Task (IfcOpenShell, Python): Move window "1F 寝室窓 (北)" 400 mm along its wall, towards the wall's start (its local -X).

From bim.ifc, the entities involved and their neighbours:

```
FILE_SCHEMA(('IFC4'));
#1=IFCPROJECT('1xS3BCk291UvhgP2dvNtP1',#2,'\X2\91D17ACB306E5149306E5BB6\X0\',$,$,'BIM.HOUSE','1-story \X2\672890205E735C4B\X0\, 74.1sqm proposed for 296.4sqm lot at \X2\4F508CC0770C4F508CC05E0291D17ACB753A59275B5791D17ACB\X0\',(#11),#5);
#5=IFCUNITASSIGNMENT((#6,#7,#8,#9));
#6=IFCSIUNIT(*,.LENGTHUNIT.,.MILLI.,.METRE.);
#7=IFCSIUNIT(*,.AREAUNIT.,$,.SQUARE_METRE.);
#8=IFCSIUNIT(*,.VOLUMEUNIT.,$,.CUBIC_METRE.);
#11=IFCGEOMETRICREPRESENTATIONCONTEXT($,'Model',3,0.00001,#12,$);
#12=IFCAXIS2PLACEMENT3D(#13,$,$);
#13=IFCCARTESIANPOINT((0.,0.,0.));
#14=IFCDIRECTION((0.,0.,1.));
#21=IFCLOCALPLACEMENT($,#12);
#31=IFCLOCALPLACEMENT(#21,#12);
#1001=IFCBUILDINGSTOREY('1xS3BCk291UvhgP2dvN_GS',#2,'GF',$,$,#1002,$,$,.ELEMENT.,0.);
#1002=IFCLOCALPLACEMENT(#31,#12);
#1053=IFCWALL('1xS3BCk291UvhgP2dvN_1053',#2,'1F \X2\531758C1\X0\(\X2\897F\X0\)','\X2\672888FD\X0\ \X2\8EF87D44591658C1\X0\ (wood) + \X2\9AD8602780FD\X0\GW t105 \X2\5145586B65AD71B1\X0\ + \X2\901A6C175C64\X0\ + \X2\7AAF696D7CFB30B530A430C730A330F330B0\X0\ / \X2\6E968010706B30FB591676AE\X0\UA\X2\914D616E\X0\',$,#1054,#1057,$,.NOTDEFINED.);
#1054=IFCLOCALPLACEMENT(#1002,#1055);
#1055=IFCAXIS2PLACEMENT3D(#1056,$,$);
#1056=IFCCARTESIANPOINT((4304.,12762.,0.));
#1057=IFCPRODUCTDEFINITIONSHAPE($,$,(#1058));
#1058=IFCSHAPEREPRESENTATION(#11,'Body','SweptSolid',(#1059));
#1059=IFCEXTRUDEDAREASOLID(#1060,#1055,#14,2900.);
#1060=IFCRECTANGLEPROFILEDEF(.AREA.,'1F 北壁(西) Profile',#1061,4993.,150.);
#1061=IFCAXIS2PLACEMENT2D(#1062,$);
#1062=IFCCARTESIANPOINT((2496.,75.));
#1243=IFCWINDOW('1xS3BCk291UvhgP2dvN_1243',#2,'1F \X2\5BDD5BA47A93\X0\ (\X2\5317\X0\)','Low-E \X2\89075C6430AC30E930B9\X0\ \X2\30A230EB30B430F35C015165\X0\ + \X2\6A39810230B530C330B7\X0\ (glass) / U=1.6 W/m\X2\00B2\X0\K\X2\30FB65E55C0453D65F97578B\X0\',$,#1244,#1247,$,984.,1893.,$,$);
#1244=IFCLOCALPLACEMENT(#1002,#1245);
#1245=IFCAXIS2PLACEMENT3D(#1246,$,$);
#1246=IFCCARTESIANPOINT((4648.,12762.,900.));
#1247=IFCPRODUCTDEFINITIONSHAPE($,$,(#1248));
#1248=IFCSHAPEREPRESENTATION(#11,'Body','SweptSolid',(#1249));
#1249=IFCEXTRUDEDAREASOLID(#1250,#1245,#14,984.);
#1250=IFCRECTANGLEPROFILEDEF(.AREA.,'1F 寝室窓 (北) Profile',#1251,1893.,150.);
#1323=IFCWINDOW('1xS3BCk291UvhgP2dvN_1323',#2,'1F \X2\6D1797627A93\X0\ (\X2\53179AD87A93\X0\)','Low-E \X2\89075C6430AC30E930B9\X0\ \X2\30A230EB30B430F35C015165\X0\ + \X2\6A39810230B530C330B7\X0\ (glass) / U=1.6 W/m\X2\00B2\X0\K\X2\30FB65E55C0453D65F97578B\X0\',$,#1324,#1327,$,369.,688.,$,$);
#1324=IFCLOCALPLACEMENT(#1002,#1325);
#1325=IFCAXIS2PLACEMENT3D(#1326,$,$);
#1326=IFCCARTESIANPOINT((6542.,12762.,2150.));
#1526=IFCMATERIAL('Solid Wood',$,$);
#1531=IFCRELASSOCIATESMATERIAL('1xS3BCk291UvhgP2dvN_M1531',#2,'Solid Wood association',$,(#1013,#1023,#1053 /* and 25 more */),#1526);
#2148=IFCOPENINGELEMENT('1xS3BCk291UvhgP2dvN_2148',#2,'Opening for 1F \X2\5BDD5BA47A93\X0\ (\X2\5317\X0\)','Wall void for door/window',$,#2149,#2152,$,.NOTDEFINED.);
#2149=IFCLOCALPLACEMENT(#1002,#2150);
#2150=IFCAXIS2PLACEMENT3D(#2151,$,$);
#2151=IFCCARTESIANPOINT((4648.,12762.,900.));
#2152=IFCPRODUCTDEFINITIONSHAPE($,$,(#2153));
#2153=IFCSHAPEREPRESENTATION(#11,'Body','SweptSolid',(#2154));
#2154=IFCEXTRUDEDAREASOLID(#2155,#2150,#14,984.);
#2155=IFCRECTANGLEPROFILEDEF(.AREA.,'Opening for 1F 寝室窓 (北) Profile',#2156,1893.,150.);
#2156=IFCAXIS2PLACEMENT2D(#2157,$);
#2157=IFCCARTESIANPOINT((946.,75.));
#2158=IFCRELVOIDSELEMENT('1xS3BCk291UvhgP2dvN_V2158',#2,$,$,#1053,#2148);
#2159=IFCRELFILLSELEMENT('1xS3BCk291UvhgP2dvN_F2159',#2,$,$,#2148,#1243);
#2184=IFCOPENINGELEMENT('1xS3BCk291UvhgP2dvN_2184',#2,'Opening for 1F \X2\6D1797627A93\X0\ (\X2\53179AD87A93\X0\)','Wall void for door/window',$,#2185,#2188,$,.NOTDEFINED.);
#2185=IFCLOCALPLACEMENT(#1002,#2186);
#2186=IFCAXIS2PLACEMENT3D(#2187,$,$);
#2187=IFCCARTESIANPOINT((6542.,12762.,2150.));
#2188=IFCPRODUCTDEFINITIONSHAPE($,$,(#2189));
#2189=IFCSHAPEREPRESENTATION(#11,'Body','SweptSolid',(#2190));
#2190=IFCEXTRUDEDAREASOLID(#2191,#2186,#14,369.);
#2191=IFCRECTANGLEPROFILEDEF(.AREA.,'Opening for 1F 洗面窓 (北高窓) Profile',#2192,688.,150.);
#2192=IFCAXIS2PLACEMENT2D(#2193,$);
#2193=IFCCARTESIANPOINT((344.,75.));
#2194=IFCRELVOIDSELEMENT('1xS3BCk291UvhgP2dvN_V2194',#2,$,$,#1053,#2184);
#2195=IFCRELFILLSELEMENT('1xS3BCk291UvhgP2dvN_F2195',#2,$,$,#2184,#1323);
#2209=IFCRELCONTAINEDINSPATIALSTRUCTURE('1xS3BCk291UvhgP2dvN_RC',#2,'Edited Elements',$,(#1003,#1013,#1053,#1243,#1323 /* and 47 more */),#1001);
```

```python
import ifcopenshell
import ifcopenshell.api.geometry
import ifcopenshell.util.placement

model = ifcopenshell.open("bim.ifc")

window = model.by_guid("1xS3BCk291UvhgP2dvN_1243")
opening = window.FillsVoids[0].RelatingOpeningElement
wall = opening.VoidsElements[0].RelatingBuildingElement

wall_matrix = ifcopenshell.util.placement.get_local_placement(wall.ObjectPlacement)
shift = wall_matrix[:3, 0] * -400.0
before = ifcopenshell.util.placement.get_local_placement(window.ObjectPlacement)[:3, 3].copy()

# The window is not placed relative to its opening, so move both.
for product in (opening, window):
    matrix = ifcopenshell.util.placement.get_local_placement(product.ObjectPlacement)
    matrix[:3, 3] += shift
    ifcopenshell.api.geometry.edit_object_placement(model, product=product, matrix=matrix, is_si=False)

after = ifcopenshell.util.placement.get_local_placement(window.ObjectPlacement)[:3, 3]
print("window moved by", (after - before).round(3) + 0.0)

model.write("bim_updated.ifc")
```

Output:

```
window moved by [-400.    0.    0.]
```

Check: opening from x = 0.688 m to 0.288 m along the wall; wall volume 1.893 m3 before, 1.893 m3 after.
